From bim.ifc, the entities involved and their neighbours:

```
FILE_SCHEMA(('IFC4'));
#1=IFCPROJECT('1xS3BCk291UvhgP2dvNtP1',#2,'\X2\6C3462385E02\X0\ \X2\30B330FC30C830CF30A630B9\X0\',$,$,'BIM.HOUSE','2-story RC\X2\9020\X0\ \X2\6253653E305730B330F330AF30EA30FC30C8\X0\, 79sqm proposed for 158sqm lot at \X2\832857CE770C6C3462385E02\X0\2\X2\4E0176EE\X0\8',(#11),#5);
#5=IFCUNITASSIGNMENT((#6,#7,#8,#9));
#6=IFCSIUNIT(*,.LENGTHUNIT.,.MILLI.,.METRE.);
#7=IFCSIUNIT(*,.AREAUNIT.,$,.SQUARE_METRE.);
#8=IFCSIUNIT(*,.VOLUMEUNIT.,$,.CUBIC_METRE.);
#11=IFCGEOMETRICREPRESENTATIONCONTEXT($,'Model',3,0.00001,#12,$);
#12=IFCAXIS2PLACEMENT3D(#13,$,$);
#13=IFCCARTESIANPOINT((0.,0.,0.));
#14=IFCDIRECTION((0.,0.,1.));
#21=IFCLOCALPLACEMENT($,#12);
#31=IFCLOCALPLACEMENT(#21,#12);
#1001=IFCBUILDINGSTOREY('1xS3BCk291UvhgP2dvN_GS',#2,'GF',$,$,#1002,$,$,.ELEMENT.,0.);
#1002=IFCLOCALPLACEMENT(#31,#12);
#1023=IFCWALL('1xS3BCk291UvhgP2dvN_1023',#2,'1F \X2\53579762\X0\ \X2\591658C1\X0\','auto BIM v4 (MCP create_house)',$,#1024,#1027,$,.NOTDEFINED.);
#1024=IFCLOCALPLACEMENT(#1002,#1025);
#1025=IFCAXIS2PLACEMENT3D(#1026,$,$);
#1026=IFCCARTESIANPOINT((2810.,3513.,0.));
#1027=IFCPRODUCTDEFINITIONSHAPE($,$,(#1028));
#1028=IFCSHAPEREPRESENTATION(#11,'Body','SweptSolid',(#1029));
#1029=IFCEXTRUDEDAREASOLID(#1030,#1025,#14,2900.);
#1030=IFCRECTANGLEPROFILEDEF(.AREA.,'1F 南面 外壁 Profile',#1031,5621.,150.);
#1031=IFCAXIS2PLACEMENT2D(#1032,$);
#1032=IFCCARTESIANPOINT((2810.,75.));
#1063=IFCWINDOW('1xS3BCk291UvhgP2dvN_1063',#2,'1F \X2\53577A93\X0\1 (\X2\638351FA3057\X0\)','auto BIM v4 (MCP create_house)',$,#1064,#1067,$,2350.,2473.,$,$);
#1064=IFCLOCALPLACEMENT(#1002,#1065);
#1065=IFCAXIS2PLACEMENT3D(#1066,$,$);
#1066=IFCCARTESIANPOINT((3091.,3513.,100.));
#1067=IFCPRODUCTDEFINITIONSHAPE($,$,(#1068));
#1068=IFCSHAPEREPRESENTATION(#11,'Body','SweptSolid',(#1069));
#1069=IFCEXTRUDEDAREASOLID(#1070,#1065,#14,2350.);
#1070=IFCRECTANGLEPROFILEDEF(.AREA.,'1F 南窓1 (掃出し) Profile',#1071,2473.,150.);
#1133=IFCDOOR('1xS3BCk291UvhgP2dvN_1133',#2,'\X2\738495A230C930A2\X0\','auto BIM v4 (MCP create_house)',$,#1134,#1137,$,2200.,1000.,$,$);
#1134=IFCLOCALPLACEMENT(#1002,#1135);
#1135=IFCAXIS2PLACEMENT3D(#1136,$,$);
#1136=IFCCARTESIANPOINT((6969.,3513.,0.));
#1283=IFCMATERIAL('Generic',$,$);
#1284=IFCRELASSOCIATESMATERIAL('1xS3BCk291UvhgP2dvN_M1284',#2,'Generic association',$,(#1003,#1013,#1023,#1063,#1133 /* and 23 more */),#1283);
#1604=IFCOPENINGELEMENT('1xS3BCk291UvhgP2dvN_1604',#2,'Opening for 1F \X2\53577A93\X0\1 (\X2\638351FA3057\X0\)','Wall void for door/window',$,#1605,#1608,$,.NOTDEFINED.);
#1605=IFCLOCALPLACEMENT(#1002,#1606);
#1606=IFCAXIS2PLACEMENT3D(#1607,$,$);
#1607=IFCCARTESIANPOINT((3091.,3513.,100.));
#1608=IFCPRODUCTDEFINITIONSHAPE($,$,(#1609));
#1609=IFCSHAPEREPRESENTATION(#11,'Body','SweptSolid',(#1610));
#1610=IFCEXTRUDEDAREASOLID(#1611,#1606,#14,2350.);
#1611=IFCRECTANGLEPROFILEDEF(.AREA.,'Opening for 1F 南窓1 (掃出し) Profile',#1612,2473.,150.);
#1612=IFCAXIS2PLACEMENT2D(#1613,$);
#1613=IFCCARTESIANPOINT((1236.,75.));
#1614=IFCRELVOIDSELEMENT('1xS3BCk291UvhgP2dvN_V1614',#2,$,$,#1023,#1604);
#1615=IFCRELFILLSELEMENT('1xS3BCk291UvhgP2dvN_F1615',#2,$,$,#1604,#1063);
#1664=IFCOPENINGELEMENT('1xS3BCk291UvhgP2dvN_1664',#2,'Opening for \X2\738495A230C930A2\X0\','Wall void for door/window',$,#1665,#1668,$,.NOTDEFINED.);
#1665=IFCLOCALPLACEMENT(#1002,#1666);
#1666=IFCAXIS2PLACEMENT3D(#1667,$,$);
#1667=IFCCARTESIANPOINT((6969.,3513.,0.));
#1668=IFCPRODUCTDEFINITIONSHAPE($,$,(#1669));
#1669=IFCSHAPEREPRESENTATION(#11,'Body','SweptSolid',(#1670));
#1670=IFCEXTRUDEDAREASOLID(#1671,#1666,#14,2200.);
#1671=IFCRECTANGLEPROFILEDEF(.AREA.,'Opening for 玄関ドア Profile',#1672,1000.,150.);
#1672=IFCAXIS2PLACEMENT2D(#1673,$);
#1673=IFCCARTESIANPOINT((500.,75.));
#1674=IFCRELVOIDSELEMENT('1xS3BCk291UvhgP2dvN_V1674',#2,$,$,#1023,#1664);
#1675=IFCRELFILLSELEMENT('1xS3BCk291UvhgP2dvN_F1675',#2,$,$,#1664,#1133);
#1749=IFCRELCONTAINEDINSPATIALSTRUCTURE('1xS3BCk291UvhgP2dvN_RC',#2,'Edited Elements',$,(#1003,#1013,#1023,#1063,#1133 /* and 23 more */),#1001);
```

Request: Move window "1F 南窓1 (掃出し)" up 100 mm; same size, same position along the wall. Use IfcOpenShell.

```python
import numpy as np
import ifcopenshell
import ifcopenshell.api.geometry
import ifcopenshell.util.placement
import ifcopenshell.util.unit

model = ifcopenshell.open("bim.ifc")
unit_scale = ifcopenshell.util.unit.calculate_unit_scale(model)

window = model.by_guid("1xS3BCk291UvhgP2dvN_1063")
opening = window.FillsVoids[0].RelatingOpeningElement
dz = 100.0

shift = np.array([0.0, 0.0, dz])
# The window is not placed relative to its opening, so move both.
for product in (opening, window):
    matrix = ifcopenshell.util.placement.get_local_placement(product.ObjectPlacement)
    matrix[:3, 3] += shift
    ifcopenshell.api.geometry.edit_object_placement(model, product=product, matrix=matrix, is_si=False)

print(f"moved by {dz * unit_scale:+.3f} m")

model.write("bim_v2.ifc")
```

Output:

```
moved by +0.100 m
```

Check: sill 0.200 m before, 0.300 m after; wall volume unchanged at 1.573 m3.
